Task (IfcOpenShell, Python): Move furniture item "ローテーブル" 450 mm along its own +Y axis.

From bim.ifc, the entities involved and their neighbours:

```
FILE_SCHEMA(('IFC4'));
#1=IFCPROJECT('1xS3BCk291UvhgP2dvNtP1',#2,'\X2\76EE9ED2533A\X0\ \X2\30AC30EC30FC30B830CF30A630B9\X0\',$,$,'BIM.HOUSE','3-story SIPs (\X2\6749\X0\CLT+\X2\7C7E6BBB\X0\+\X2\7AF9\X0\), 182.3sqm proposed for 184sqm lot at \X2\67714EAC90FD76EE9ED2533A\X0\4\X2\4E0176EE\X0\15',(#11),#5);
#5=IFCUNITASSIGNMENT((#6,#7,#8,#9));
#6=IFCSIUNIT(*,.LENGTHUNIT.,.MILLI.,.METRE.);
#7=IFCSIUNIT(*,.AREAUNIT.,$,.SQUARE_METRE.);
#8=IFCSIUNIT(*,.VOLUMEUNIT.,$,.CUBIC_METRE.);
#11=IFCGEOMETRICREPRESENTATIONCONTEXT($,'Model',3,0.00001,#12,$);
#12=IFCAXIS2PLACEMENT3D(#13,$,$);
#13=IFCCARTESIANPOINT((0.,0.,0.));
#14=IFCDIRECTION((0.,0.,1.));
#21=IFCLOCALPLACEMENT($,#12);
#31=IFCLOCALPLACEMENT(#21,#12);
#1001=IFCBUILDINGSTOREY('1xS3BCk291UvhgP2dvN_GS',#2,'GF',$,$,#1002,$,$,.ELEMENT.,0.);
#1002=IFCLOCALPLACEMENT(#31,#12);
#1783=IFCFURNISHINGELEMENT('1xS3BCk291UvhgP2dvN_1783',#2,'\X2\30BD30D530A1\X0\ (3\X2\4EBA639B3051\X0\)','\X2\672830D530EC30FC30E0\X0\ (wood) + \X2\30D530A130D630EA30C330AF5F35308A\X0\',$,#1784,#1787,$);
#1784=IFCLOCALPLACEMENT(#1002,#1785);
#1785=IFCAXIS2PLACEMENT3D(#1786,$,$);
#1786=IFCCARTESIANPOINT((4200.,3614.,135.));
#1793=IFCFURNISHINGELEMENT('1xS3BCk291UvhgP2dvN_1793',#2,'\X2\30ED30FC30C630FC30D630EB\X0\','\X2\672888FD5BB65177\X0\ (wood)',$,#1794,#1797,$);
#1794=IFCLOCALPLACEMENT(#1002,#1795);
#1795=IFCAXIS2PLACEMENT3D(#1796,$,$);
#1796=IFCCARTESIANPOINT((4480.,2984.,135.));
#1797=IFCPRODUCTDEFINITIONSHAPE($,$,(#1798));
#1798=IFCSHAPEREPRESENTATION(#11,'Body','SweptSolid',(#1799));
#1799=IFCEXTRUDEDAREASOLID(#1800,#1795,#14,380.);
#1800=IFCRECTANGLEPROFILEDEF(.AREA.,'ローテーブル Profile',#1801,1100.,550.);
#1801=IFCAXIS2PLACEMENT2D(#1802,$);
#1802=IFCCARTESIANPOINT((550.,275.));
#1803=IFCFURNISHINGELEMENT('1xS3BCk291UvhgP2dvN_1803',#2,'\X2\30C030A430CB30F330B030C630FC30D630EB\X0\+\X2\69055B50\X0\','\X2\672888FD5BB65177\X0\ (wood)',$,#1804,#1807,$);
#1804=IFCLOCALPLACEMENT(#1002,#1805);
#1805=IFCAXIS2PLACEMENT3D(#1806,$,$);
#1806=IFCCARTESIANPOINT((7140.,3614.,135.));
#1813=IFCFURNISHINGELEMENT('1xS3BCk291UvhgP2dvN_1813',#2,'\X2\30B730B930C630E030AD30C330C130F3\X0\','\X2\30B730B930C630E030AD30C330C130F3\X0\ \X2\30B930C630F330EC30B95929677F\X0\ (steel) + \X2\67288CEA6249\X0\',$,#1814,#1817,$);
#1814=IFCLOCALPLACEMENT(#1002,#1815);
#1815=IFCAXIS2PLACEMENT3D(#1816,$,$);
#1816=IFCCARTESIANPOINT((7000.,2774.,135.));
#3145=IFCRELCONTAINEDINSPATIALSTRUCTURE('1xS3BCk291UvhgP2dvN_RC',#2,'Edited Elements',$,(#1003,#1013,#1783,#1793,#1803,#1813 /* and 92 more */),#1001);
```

```python
import ifcopenshell
import ifcopenshell.api.geometry
import ifcopenshell.util.placement
import ifcopenshell.util.unit

model = ifcopenshell.open("bim.ifc")
unit_scale = ifcopenshell.util.unit.calculate_unit_scale(model)

item = model.by_guid("1xS3BCk291UvhgP2dvN_1793")
matrix = ifcopenshell.util.placement.get_local_placement(item.ObjectPlacement)
matrix[:3, 3] += matrix[:3, 1] * 0.45 / unit_scale
ifcopenshell.api.geometry.edit_object_placement(model, product=item, matrix=matrix, is_si=False)

print(ifcopenshell.util.placement.get_local_placement(item.ObjectPlacement).round(3) + 0.0)

model.write("bim_rev.ifc")
```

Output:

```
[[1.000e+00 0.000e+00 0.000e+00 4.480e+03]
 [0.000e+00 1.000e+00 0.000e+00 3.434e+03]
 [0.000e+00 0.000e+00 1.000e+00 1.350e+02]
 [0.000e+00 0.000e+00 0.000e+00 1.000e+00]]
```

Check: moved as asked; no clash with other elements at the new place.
